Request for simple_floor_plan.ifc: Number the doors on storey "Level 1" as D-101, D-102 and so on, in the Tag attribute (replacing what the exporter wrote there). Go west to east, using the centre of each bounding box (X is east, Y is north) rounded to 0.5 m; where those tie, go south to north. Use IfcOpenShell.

First a look at what the model holds.

```python
import ifcopenshell
import ifcopenshell.util.element
import ifcopenshell.util.placement

model = ifcopenshell.open("simple_floor_plan.ifc")
print(model.schema)
storey = next(s for s in model.by_type("IfcBuildingStorey") if s.Name == "Level 1")
doors = [e for e in ifcopenshell.util.element.get_decomposition(storey) if e.is_a("IfcDoor")]
for e in sorted(doors, key=lambda e: e.id()):
    origin = ifcopenshell.util.placement.get_local_placement(e.ObjectPlacement)[:3, 3]
    print(e.id(), e.Tag, e.Name, origin.round(2) + 0.0, sep=" | ")
```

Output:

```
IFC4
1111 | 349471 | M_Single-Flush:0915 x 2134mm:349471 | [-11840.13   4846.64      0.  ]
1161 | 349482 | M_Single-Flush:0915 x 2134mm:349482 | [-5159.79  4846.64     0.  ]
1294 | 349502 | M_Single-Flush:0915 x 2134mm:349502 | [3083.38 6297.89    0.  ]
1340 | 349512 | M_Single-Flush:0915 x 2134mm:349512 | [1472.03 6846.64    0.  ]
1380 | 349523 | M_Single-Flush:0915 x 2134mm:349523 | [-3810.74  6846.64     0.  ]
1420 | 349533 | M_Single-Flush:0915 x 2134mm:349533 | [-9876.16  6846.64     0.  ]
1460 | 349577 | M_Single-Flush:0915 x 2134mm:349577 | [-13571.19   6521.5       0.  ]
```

```python
import ifcopenshell
import ifcopenshell.geom
import ifcopenshell.util.element
import ifcopenshell.util.shape

model = ifcopenshell.open("simple_floor_plan.ifc")
settings = ifcopenshell.geom.settings()
settings.set("use-world-coords", True)


def centre(element):
    shape = ifcopenshell.geom.create_shape(settings, element)
    return ifcopenshell.util.shape.get_bbox_centroid(shape.geometry)


storey = next(s for s in model.by_type("IfcBuildingStorey") if s.Name == "Level 1")
doors = [e for e in ifcopenshell.util.element.get_decomposition(storey) if e.is_a("IfcDoor")]

# Insertion points can sit at a corner or the storey origin, so sort by the geometry (in metres).
centres = {e: centre(e) for e in doors}
doors.sort(key=lambda e: (round(centres[e][0] / 0.5), centres[e][1]))

for i, e in enumerate(doors, start=1):
    number = f"D-1{i:02d}"
    e.Tag = number
    print(e.id(), number)

model.write("simple_floor_plan-out.ifc")
```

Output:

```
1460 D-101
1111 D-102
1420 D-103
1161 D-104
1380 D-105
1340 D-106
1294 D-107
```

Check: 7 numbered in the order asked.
